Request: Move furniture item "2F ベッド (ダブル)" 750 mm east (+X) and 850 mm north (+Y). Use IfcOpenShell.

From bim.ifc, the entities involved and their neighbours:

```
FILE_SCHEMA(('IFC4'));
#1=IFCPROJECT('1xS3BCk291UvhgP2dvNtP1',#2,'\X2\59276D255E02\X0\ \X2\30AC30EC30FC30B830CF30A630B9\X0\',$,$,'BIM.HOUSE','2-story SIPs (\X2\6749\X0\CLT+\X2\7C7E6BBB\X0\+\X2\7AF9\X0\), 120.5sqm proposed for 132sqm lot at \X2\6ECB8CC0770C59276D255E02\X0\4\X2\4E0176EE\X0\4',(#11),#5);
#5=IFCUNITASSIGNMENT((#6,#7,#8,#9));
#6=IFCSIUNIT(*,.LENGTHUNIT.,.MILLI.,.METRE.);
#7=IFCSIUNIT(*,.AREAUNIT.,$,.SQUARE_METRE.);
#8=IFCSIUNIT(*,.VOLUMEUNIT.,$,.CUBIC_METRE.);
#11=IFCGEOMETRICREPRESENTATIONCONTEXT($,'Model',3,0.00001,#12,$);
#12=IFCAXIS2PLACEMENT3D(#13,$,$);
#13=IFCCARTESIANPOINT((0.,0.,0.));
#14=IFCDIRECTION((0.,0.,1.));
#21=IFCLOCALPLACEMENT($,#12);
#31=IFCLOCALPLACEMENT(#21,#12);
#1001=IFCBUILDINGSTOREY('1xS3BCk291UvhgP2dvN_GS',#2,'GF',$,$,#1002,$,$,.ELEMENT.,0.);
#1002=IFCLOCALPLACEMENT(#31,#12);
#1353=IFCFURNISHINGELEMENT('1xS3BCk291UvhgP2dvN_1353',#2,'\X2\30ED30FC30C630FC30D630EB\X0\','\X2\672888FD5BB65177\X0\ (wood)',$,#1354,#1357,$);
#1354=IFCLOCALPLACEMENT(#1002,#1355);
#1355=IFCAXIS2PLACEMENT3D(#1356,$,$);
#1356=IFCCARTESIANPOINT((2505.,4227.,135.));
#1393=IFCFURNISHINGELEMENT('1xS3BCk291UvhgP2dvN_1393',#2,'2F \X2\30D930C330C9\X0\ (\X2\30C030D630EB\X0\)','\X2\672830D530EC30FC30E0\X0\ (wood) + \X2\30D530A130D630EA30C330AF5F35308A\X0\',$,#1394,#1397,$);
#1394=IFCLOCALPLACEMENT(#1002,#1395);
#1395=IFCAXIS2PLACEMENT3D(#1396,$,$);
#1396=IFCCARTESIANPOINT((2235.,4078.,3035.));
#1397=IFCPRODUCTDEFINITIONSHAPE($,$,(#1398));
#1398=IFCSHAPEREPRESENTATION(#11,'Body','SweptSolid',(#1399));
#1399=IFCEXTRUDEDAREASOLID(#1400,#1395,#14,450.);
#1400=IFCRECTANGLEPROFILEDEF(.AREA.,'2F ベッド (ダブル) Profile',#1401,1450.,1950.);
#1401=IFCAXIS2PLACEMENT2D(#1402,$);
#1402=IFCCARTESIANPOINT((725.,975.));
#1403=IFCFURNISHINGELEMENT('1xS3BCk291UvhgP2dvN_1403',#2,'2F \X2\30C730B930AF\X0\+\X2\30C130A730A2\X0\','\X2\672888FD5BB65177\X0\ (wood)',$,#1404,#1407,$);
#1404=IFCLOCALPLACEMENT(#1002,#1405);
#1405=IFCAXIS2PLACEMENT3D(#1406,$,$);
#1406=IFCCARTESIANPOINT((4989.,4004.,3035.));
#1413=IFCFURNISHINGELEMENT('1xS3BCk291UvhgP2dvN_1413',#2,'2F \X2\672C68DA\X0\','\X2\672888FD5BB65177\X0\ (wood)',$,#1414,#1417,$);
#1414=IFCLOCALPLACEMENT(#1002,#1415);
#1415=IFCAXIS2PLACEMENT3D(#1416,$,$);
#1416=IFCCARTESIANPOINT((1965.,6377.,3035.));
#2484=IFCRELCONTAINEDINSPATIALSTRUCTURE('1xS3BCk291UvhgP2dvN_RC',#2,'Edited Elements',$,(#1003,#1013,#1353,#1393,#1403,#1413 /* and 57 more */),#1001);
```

```python
import ifcopenshell
import ifcopenshell.api.geometry
import ifcopenshell.util.placement
import ifcopenshell.util.unit

model = ifcopenshell.open("bim.ifc")
unit_scale = ifcopenshell.util.unit.calculate_unit_scale(model)

item = model.by_guid("1xS3BCk291UvhgP2dvN_1393")
matrix = ifcopenshell.util.placement.get_local_placement(item.ObjectPlacement)
matrix[0, 3] += 0.75 / unit_scale
matrix[1, 3] += 0.85 / unit_scale
ifcopenshell.api.geometry.edit_object_placement(model, product=item, matrix=matrix, is_si=False)

print(ifcopenshell.util.placement.get_local_placement(item.ObjectPlacement).round(3) + 0.0)

model.write("bim-out.ifc")
```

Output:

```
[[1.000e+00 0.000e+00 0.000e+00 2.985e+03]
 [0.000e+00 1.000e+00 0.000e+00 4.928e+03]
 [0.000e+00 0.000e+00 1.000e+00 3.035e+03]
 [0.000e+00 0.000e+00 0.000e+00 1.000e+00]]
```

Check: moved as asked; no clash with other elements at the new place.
